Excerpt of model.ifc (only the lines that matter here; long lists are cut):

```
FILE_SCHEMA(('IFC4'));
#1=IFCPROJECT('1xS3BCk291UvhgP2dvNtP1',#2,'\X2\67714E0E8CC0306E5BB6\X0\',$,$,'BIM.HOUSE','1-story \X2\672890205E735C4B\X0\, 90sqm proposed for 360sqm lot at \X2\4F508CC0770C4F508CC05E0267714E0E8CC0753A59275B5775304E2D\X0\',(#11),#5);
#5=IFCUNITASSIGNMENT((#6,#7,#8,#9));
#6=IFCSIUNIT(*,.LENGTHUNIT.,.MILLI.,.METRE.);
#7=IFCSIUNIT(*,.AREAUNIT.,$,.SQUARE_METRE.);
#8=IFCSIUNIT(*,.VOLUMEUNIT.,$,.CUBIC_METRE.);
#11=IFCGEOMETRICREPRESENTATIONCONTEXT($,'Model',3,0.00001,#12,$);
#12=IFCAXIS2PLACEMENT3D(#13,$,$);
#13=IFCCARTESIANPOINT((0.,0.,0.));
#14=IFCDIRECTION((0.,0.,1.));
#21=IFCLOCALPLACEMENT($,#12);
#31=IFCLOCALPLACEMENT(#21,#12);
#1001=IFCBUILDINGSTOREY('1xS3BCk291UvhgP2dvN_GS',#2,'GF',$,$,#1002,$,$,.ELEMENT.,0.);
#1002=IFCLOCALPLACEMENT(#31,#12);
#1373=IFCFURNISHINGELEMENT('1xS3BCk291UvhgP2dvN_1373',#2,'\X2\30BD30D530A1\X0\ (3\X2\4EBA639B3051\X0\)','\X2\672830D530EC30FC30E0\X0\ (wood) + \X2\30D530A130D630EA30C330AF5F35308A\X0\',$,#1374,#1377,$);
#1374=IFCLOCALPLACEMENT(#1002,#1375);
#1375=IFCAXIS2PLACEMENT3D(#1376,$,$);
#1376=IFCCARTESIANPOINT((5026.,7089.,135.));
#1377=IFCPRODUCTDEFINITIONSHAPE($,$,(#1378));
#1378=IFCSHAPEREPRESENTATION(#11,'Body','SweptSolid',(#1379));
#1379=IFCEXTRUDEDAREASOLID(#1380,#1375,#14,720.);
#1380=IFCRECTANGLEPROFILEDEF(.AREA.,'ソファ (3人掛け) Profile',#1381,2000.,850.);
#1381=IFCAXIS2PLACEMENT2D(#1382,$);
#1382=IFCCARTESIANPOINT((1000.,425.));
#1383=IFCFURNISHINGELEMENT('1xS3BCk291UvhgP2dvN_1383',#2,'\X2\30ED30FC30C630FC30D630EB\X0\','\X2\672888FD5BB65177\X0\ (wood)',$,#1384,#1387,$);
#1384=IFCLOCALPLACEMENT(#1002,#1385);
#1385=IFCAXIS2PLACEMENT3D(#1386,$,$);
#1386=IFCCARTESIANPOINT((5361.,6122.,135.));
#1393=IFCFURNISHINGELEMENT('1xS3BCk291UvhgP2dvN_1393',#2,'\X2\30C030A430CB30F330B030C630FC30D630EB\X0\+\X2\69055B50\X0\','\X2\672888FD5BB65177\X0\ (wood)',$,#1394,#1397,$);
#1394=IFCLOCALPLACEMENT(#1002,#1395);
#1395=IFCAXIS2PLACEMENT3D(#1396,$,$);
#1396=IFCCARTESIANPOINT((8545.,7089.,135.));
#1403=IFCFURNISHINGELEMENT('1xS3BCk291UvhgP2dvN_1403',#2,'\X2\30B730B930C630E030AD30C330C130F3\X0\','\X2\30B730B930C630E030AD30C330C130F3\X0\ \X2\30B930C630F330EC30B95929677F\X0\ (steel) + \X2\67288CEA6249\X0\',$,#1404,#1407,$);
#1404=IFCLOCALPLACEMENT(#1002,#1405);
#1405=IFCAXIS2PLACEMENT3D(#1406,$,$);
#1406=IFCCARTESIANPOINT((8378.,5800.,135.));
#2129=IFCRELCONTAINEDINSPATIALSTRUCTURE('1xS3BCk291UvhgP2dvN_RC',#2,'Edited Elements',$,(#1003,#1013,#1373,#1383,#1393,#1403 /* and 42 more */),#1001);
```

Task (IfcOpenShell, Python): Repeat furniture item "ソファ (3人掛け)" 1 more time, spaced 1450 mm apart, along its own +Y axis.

```python
import ifcopenshell
import ifcopenshell.api.geometry
import ifcopenshell.api.root
import ifcopenshell.util.element
import ifcopenshell.util.placement
import ifcopenshell.util.unit

model = ifcopenshell.open("model.ifc")
unit_scale = ifcopenshell.util.unit.calculate_unit_scale(model)


def reuse_history(source, copy):
    """copy_class also copies each property set's owner history, people and application; keep the originals."""
    for rel in copy.IsDefinedBy:
        if rel.is_a("IfcRelDefinesByProperties") and (history := rel.RelatingPropertyDefinition.OwnerHistory):
            rel.RelatingPropertyDefinition.OwnerHistory = source.OwnerHistory
            ifcopenshell.util.element.remove_deep2(model, history)


source = model.by_id(1373)
base = ifcopenshell.util.placement.get_local_placement(source.ObjectPlacement)
step = base[:3, 1] * 1.45 / unit_scale

for i in range(1, 2):
    copy = ifcopenshell.api.root.copy_class(model, product=source)
    copy.Representation = ifcopenshell.util.element.copy_deep(
        model, source.Representation, exclude=["IfcGeometricRepresentationContext", "IfcRepresentationMap"]
    )
    reuse_history(source, copy)
    matrix = base.copy()
    matrix[:3, 3] += i * step
    print("added at", matrix[:3, 3].round(3) + 0.0)
    ifcopenshell.api.geometry.edit_object_placement(model, product=copy, matrix=matrix, is_si=False)

model.write("model_updated.ifc")
```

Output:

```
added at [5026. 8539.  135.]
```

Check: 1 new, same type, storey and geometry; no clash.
